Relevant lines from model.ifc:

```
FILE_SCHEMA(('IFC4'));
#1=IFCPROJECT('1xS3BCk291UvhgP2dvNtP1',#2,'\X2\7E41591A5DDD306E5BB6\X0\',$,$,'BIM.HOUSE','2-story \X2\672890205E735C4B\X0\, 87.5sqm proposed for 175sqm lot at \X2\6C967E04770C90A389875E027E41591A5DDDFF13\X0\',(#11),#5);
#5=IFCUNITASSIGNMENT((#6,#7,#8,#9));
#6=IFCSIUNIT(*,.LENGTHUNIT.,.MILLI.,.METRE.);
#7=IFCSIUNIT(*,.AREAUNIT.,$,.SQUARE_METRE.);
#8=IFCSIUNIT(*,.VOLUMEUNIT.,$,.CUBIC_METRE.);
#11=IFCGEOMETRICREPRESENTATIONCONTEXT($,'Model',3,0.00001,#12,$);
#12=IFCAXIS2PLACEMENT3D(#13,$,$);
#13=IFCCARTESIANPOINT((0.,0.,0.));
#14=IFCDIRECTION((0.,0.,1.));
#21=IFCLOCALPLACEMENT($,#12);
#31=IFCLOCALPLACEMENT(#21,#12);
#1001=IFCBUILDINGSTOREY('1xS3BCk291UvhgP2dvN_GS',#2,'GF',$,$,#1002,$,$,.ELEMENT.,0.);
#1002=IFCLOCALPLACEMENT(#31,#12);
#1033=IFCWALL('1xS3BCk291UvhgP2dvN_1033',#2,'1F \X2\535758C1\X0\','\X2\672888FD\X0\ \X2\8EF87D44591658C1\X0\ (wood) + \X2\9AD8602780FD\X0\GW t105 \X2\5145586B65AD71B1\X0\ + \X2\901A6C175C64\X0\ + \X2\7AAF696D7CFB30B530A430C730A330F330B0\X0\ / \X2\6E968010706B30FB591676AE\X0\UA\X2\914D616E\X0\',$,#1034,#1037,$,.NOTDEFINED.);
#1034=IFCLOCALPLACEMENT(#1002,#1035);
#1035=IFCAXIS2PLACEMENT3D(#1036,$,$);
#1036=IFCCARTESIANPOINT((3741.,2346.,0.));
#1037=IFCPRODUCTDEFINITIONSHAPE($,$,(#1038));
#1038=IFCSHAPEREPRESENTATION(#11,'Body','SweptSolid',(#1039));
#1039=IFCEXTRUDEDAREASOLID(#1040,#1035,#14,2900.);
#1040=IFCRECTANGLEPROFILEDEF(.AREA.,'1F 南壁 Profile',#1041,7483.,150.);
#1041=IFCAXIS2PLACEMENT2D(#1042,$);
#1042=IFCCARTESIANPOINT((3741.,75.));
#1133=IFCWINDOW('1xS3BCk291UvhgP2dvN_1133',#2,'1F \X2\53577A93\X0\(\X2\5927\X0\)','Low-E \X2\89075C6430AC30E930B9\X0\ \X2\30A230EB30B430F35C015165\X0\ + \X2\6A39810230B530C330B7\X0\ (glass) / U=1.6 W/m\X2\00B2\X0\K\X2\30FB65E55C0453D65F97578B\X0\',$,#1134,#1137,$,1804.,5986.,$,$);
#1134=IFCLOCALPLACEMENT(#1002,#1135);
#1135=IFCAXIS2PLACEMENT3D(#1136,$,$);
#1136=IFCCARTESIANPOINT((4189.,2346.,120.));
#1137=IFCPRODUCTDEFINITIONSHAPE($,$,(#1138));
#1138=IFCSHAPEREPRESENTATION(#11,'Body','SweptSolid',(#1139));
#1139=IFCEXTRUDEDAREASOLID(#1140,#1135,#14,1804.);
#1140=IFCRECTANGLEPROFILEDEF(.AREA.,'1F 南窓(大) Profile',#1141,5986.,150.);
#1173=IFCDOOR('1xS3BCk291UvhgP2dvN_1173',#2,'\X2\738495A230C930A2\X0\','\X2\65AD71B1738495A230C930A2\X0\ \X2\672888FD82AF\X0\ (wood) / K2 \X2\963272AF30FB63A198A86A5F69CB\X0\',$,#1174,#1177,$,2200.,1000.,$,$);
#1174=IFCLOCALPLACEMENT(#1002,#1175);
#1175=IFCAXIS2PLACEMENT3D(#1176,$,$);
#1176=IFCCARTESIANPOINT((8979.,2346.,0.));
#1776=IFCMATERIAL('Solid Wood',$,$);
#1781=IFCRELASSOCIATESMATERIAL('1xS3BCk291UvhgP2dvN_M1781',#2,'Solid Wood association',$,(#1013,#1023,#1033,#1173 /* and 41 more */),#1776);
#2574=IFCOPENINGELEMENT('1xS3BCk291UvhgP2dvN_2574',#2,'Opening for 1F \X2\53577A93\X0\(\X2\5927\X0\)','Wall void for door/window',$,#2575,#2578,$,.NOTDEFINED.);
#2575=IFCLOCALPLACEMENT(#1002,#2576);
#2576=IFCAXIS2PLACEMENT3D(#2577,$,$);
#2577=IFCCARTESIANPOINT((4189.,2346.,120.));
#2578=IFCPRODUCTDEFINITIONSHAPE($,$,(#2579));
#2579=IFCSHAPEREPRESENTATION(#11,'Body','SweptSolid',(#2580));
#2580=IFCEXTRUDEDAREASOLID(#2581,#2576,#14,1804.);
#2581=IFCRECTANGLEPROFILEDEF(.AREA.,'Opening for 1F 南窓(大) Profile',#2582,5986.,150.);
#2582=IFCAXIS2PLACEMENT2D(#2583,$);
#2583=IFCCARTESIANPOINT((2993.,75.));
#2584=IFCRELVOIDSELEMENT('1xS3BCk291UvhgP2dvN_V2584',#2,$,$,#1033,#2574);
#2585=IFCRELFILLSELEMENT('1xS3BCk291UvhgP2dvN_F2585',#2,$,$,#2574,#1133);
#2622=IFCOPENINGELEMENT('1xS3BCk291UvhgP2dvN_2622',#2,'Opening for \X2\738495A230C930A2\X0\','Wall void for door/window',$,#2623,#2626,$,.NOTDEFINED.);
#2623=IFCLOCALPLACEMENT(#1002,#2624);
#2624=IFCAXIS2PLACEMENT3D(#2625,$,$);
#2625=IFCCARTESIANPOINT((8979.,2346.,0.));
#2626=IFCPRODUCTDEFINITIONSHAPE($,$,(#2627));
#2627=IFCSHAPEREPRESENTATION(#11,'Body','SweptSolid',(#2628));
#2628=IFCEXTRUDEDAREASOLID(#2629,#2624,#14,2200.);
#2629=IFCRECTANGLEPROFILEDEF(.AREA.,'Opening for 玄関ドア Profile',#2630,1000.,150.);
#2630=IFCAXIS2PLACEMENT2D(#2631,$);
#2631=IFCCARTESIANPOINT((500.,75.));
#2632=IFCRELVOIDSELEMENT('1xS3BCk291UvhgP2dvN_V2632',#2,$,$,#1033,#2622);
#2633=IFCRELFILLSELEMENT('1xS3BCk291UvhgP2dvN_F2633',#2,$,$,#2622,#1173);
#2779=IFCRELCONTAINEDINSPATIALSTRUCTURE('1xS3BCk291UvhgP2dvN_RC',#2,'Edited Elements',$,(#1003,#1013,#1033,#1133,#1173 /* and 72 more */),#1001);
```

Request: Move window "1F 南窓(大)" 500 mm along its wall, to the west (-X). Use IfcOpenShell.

```python
import ifcopenshell
import ifcopenshell.api.geometry
import ifcopenshell.util.placement

model = ifcopenshell.open("model.ifc")

window = model.by_guid("1xS3BCk291UvhgP2dvN_1133")
opening = window.FillsVoids[0].RelatingOpeningElement
wall = opening.VoidsElements[0].RelatingBuildingElement

wall_matrix = ifcopenshell.util.placement.get_local_placement(wall.ObjectPlacement)
shift = wall_matrix[:3, 0] * -500.0
before = ifcopenshell.util.placement.get_local_placement(window.ObjectPlacement)[:3, 3].copy()

# The window is not placed relative to its opening, so move both.
for product in (opening, window):
    matrix = ifcopenshell.util.placement.get_local_placement(product.ObjectPlacement)
    matrix[:3, 3] += shift
    ifcopenshell.api.geometry.edit_object_placement(model, product=product, matrix=matrix, is_si=False)

after = ifcopenshell.util.placement.get_local_placement(window.ObjectPlacement)[:3, 3]
print("window moved by", (after - before).round(3) + 0.0)

model.write("model-out.ifc")
```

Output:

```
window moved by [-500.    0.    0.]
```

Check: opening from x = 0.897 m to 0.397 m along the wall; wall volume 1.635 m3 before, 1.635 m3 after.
